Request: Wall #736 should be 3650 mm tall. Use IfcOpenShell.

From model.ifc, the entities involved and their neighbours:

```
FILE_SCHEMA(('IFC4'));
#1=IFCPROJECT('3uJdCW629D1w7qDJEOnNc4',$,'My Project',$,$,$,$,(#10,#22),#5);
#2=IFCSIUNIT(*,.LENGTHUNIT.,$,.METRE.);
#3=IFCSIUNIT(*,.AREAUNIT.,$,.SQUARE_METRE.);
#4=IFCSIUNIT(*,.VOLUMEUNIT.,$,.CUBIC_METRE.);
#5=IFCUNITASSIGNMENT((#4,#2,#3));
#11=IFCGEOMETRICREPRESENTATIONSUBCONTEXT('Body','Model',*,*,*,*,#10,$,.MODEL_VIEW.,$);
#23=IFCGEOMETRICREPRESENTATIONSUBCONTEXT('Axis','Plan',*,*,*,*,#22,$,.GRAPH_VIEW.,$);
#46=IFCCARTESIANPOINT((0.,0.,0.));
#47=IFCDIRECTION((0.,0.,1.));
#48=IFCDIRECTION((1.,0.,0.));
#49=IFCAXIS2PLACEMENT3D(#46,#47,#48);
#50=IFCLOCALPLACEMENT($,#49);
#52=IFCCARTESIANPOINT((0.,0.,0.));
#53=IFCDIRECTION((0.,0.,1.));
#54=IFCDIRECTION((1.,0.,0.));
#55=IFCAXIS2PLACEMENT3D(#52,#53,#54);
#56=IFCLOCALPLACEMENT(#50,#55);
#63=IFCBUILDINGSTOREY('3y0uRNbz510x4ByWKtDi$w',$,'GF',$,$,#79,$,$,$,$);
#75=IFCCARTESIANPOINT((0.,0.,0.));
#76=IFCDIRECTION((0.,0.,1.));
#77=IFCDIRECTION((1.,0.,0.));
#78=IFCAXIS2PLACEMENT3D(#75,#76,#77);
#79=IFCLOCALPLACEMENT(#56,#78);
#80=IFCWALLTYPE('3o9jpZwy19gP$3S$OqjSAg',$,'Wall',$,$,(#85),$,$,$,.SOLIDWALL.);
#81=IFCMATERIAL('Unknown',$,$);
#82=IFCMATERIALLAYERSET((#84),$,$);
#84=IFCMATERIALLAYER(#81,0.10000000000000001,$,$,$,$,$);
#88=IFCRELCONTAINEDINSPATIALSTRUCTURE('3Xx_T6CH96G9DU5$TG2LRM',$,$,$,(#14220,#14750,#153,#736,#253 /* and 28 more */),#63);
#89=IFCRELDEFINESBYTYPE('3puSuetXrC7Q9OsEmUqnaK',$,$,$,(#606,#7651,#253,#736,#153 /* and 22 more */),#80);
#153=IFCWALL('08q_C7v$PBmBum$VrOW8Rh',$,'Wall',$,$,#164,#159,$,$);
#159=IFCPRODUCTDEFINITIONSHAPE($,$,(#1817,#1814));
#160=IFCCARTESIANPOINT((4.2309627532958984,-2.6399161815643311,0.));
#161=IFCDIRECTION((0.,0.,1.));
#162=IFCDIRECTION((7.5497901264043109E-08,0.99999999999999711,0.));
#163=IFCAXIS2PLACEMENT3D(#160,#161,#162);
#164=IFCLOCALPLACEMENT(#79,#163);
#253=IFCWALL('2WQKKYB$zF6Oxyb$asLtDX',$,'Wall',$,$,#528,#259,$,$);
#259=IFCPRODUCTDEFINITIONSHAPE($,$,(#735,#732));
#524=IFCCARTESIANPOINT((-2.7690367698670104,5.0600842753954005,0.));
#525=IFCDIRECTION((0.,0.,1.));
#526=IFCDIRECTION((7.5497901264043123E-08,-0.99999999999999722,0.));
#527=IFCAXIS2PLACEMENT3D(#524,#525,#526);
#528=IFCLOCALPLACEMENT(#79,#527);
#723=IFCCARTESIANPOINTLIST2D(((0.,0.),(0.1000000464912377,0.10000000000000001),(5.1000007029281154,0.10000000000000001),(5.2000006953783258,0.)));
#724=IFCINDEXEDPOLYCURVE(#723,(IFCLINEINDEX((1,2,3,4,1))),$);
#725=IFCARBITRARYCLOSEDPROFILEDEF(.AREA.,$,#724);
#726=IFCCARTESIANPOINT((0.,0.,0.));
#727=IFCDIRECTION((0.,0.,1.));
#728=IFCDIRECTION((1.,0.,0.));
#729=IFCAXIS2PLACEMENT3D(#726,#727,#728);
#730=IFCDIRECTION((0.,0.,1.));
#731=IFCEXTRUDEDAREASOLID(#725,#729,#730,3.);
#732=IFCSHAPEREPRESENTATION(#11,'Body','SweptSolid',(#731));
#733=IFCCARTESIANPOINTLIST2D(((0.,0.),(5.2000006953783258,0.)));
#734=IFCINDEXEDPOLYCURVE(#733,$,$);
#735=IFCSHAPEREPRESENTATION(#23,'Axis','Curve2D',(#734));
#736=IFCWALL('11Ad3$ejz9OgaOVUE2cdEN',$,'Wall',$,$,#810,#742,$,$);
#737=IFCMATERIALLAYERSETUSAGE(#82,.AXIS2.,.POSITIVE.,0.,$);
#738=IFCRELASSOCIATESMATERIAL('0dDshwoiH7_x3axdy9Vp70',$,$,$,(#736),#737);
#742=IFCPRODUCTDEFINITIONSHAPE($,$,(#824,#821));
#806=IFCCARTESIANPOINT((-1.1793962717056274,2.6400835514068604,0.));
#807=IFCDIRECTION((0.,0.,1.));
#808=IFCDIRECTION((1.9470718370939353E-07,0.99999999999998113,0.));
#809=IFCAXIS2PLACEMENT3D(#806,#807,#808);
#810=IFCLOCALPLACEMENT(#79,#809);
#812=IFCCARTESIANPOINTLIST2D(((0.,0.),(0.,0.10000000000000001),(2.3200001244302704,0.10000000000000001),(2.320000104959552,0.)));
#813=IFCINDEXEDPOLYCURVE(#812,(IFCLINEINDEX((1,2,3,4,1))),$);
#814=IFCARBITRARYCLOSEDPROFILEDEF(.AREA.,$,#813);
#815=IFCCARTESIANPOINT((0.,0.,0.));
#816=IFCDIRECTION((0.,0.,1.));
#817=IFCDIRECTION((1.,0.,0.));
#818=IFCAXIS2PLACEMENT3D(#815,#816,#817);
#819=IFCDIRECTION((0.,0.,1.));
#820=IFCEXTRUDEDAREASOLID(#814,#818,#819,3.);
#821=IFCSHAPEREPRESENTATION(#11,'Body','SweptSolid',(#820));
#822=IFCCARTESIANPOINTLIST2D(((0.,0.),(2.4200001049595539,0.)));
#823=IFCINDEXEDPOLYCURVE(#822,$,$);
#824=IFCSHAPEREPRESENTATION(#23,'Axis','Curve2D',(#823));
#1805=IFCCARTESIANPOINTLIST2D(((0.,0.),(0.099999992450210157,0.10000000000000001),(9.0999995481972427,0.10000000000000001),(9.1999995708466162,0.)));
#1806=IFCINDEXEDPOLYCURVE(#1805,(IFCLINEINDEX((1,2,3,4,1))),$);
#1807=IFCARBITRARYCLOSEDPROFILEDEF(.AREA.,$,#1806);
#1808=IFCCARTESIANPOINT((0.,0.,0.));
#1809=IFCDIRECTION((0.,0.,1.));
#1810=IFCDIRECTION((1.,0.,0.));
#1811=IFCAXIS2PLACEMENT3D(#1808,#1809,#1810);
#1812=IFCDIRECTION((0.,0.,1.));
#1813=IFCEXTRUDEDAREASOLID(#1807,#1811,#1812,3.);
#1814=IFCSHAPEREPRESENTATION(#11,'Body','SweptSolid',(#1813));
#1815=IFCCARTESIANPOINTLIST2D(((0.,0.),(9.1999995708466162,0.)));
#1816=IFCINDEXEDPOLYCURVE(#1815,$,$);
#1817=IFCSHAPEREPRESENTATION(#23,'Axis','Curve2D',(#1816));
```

```python
import ifcopenshell
import ifcopenshell.geom
import ifcopenshell.util.representation
import ifcopenshell.util.shape
import ifcopenshell.util.unit

model = ifcopenshell.open("model.ifc")
unit_scale = ifcopenshell.util.unit.calculate_unit_scale(model)
settings = ifcopenshell.geom.settings()


def volume(element):
    """Net volume in cubic metres, openings subtracted."""
    shape = ifcopenshell.geom.create_shape(settings, element)
    return ifcopenshell.util.shape.get_volume(shape.geometry)


wall = model.by_guid("11Ad3$ejz9OgaOVUE2cdEN")
before = volume(wall)

body = ifcopenshell.util.representation.get_representation(wall, "Model", "Body")
solid = body.Items[0]
old_height = solid.Depth
solid.Depth = 3.65 / unit_scale
after = volume(wall)

print(f"height {old_height:g} -> {solid.Depth:g}, volume {before:.3f} -> {after:.3f} m3")

model.write("model_v2.ifc")
```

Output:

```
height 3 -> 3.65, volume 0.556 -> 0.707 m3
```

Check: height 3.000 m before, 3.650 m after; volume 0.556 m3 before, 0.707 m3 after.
